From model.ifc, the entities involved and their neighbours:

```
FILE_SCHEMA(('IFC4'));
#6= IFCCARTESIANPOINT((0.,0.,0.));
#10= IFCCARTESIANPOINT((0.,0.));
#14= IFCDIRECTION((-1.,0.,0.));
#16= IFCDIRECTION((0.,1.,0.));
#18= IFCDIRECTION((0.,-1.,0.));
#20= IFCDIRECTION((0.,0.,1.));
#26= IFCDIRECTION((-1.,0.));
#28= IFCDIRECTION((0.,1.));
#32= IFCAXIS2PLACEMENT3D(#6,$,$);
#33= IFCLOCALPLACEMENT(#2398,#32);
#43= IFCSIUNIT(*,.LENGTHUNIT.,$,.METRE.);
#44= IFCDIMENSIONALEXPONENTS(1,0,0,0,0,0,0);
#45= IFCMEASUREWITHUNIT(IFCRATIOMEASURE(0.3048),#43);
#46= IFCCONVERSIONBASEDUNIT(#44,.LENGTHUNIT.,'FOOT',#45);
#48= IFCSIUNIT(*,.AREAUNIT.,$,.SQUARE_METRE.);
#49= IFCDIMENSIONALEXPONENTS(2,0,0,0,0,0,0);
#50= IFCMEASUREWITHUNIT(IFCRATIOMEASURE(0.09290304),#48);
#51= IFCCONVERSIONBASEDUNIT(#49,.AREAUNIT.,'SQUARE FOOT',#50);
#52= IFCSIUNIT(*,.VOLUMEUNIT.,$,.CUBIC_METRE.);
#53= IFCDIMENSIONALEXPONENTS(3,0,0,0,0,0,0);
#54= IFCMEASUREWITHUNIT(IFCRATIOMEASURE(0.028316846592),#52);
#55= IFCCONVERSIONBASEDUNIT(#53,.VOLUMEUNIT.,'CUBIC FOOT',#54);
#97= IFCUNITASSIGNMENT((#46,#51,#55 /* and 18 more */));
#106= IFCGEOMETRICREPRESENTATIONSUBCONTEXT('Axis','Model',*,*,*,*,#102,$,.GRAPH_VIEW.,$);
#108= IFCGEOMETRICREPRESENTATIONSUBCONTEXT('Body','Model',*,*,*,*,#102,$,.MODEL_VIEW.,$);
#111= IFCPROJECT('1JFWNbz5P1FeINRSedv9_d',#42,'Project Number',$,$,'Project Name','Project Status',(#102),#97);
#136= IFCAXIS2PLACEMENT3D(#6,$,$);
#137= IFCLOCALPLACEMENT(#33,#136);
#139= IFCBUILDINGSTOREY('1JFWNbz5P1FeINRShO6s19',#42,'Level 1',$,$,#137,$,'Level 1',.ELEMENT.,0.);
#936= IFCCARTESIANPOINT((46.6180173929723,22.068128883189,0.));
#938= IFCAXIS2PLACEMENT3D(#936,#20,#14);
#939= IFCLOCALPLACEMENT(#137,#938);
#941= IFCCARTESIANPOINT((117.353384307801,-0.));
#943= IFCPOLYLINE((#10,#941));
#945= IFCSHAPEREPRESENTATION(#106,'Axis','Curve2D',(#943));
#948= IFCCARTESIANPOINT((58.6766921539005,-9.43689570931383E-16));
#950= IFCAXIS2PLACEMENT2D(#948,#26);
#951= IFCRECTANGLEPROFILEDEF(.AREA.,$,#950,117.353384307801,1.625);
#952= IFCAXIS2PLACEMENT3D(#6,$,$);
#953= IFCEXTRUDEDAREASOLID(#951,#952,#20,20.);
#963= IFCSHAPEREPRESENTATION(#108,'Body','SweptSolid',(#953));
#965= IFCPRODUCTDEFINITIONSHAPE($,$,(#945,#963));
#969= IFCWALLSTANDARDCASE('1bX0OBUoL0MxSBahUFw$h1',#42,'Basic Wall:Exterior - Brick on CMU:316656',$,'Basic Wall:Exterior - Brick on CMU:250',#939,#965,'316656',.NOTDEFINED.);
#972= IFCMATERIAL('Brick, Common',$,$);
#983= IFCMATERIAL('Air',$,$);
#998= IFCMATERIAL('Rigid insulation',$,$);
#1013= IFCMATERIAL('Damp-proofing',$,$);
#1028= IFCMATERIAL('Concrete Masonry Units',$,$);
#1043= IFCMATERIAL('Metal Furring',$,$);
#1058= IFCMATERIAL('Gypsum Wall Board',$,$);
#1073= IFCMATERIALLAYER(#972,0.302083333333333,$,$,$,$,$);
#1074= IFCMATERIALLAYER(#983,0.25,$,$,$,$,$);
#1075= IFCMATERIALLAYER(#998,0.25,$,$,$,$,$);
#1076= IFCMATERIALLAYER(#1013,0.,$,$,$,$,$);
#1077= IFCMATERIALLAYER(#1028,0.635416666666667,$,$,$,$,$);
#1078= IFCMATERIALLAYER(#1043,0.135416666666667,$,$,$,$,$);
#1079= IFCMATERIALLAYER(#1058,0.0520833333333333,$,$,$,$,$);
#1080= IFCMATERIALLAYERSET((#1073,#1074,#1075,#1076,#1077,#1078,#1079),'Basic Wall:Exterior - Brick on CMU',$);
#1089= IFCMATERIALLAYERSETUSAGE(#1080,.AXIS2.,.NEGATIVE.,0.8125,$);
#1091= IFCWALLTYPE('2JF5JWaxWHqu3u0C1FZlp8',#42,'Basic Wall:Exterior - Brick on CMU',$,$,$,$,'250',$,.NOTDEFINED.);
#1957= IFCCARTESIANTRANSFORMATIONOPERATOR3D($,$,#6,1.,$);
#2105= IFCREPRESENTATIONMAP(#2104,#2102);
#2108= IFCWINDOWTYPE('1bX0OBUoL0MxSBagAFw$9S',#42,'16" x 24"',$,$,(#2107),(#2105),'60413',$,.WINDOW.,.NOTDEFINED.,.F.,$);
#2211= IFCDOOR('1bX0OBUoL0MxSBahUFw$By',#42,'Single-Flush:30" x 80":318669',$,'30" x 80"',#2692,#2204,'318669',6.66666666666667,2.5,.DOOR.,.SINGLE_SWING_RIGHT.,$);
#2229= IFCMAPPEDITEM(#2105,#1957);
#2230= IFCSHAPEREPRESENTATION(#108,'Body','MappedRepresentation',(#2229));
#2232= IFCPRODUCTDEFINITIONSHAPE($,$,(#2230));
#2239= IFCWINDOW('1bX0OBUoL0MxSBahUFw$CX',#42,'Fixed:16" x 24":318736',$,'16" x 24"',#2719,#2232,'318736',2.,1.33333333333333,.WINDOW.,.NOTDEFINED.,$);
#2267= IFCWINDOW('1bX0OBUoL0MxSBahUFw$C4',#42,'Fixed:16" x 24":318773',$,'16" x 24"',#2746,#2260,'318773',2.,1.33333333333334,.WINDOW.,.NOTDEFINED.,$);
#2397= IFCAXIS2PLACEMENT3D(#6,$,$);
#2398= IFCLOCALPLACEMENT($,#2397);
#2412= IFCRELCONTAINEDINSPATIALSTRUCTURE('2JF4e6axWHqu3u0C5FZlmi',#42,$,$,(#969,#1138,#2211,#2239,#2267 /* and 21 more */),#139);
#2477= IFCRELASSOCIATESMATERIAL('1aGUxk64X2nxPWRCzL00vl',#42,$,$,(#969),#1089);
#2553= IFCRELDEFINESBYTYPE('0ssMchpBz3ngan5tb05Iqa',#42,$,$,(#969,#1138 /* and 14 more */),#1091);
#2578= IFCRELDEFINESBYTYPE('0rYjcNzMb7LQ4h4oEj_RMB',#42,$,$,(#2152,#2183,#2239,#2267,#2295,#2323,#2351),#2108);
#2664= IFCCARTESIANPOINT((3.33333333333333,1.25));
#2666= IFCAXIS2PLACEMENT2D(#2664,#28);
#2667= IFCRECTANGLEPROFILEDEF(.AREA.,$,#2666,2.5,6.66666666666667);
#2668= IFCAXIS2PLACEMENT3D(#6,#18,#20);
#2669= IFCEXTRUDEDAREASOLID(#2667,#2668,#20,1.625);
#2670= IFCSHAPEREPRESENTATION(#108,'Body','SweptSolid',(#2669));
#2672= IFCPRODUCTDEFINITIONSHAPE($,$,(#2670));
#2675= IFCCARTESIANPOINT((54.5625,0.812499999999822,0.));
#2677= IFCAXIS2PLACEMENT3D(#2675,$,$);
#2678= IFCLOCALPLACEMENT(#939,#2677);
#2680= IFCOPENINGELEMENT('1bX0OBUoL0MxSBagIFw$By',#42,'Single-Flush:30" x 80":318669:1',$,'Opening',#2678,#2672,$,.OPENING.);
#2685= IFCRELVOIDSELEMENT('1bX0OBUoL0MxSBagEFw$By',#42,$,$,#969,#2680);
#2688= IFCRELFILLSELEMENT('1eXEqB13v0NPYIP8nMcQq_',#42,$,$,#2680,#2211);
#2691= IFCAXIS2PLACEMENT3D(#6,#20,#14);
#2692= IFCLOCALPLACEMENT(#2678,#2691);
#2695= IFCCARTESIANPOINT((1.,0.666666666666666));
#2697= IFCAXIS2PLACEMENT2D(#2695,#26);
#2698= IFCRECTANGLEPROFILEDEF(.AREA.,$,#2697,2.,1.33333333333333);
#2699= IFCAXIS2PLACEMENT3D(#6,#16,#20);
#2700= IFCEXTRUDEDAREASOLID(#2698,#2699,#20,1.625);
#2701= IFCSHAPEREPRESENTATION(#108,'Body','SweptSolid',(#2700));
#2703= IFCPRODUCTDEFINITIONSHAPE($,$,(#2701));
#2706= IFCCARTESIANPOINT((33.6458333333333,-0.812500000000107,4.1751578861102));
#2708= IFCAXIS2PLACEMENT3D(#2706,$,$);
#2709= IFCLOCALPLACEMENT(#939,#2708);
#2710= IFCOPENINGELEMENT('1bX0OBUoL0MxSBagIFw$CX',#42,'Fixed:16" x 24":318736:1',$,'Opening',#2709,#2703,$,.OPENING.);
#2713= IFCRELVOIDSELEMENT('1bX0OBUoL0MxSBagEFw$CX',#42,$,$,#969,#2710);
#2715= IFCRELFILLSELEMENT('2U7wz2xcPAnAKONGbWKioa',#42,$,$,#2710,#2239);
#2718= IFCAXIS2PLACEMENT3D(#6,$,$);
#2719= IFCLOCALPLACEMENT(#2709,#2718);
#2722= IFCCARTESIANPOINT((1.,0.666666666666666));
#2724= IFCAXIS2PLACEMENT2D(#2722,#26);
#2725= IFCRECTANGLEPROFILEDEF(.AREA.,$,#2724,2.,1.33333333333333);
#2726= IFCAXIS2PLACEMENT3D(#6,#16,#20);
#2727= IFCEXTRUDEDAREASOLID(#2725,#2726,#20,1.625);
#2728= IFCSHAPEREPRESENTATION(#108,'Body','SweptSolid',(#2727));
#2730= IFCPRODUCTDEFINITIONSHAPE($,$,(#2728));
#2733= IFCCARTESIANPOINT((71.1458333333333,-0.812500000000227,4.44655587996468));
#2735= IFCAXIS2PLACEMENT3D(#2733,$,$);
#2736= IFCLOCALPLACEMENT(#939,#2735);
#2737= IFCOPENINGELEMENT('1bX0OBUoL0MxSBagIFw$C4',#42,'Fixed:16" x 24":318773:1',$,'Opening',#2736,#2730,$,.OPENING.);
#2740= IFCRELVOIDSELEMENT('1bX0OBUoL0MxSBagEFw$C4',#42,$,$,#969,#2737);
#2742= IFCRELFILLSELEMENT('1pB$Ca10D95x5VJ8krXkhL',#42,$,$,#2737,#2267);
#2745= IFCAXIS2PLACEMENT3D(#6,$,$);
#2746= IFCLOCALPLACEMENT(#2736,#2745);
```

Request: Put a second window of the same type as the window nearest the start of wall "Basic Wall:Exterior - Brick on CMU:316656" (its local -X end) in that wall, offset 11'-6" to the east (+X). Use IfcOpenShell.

```python
import ifcopenshell
import ifcopenshell.api.feature
import ifcopenshell.api.geometry
import ifcopenshell.api.root
import ifcopenshell.geom
import ifcopenshell.util.element
import ifcopenshell.util.placement
import ifcopenshell.util.shape
import ifcopenshell.util.unit

model = ifcopenshell.open("model.ifc")
unit_scale = ifcopenshell.util.unit.calculate_unit_scale(model)
settings = ifcopenshell.geom.settings()


def volume(element):
    """Net volume in cubic metres, openings subtracted."""
    shape = ifcopenshell.geom.create_shape(settings, element)
    return ifcopenshell.util.shape.get_volume(shape.geometry)


def reuse_history(source, copy):
    """copy_class also copies each property set's owner history, people and application; keep the originals."""
    for rel in copy.IsDefinedBy:
        if rel.is_a("IfcRelDefinesByProperties") and (history := rel.RelatingPropertyDefinition.OwnerHistory):
            rel.RelatingPropertyDefinition.OwnerHistory = source.OwnerHistory
            ifcopenshell.util.element.remove_deep2(model, history)


window = model.by_id(2239)
opening = window.FillsVoids[0].RelatingOpeningElement
wall = opening.VoidsElements[0].RelatingBuildingElement
before = volume(wall)
shift = ifcopenshell.util.placement.get_local_placement(wall.ObjectPlacement)[:3, 0] * -138 * 0.0254 / unit_scale

# copy_class copies the void relationship, type, container and properties, but no geometry.
new_opening = ifcopenshell.api.root.copy_class(model, product=opening)
new_opening.Representation = ifcopenshell.util.element.copy_deep(
    model, opening.Representation, exclude=["IfcGeometricRepresentationContext", "IfcRepresentationMap"]
)
new_opening.Name = 'Fixed:16" x 24"'
new_window = ifcopenshell.api.root.copy_class(model, product=window)
new_window.Representation = ifcopenshell.util.element.copy_deep(
    model, window.Representation, exclude=["IfcGeometricRepresentationContext", "IfcRepresentationMap"]
)
new_window.Name = 'Fixed:16" x 24"'
new_window.Tag = None
reuse_history(window, new_window)
ifcopenshell.api.feature.add_filling(model, opening=new_opening, element=new_window)

for old, new in ((opening, new_opening), (window, new_window)):
    matrix = ifcopenshell.util.placement.get_local_placement(old.ObjectPlacement)
    matrix[:3, 3] += shift
    ifcopenshell.api.geometry.edit_object_placement(model, product=new, matrix=matrix, is_si=False)

after = volume(wall)

print(f"wall volume {before:.3f} -> {after:.3f} m3")

model.write("model-out.ifc")
```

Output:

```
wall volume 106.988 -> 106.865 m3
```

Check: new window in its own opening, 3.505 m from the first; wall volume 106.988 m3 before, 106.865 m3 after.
